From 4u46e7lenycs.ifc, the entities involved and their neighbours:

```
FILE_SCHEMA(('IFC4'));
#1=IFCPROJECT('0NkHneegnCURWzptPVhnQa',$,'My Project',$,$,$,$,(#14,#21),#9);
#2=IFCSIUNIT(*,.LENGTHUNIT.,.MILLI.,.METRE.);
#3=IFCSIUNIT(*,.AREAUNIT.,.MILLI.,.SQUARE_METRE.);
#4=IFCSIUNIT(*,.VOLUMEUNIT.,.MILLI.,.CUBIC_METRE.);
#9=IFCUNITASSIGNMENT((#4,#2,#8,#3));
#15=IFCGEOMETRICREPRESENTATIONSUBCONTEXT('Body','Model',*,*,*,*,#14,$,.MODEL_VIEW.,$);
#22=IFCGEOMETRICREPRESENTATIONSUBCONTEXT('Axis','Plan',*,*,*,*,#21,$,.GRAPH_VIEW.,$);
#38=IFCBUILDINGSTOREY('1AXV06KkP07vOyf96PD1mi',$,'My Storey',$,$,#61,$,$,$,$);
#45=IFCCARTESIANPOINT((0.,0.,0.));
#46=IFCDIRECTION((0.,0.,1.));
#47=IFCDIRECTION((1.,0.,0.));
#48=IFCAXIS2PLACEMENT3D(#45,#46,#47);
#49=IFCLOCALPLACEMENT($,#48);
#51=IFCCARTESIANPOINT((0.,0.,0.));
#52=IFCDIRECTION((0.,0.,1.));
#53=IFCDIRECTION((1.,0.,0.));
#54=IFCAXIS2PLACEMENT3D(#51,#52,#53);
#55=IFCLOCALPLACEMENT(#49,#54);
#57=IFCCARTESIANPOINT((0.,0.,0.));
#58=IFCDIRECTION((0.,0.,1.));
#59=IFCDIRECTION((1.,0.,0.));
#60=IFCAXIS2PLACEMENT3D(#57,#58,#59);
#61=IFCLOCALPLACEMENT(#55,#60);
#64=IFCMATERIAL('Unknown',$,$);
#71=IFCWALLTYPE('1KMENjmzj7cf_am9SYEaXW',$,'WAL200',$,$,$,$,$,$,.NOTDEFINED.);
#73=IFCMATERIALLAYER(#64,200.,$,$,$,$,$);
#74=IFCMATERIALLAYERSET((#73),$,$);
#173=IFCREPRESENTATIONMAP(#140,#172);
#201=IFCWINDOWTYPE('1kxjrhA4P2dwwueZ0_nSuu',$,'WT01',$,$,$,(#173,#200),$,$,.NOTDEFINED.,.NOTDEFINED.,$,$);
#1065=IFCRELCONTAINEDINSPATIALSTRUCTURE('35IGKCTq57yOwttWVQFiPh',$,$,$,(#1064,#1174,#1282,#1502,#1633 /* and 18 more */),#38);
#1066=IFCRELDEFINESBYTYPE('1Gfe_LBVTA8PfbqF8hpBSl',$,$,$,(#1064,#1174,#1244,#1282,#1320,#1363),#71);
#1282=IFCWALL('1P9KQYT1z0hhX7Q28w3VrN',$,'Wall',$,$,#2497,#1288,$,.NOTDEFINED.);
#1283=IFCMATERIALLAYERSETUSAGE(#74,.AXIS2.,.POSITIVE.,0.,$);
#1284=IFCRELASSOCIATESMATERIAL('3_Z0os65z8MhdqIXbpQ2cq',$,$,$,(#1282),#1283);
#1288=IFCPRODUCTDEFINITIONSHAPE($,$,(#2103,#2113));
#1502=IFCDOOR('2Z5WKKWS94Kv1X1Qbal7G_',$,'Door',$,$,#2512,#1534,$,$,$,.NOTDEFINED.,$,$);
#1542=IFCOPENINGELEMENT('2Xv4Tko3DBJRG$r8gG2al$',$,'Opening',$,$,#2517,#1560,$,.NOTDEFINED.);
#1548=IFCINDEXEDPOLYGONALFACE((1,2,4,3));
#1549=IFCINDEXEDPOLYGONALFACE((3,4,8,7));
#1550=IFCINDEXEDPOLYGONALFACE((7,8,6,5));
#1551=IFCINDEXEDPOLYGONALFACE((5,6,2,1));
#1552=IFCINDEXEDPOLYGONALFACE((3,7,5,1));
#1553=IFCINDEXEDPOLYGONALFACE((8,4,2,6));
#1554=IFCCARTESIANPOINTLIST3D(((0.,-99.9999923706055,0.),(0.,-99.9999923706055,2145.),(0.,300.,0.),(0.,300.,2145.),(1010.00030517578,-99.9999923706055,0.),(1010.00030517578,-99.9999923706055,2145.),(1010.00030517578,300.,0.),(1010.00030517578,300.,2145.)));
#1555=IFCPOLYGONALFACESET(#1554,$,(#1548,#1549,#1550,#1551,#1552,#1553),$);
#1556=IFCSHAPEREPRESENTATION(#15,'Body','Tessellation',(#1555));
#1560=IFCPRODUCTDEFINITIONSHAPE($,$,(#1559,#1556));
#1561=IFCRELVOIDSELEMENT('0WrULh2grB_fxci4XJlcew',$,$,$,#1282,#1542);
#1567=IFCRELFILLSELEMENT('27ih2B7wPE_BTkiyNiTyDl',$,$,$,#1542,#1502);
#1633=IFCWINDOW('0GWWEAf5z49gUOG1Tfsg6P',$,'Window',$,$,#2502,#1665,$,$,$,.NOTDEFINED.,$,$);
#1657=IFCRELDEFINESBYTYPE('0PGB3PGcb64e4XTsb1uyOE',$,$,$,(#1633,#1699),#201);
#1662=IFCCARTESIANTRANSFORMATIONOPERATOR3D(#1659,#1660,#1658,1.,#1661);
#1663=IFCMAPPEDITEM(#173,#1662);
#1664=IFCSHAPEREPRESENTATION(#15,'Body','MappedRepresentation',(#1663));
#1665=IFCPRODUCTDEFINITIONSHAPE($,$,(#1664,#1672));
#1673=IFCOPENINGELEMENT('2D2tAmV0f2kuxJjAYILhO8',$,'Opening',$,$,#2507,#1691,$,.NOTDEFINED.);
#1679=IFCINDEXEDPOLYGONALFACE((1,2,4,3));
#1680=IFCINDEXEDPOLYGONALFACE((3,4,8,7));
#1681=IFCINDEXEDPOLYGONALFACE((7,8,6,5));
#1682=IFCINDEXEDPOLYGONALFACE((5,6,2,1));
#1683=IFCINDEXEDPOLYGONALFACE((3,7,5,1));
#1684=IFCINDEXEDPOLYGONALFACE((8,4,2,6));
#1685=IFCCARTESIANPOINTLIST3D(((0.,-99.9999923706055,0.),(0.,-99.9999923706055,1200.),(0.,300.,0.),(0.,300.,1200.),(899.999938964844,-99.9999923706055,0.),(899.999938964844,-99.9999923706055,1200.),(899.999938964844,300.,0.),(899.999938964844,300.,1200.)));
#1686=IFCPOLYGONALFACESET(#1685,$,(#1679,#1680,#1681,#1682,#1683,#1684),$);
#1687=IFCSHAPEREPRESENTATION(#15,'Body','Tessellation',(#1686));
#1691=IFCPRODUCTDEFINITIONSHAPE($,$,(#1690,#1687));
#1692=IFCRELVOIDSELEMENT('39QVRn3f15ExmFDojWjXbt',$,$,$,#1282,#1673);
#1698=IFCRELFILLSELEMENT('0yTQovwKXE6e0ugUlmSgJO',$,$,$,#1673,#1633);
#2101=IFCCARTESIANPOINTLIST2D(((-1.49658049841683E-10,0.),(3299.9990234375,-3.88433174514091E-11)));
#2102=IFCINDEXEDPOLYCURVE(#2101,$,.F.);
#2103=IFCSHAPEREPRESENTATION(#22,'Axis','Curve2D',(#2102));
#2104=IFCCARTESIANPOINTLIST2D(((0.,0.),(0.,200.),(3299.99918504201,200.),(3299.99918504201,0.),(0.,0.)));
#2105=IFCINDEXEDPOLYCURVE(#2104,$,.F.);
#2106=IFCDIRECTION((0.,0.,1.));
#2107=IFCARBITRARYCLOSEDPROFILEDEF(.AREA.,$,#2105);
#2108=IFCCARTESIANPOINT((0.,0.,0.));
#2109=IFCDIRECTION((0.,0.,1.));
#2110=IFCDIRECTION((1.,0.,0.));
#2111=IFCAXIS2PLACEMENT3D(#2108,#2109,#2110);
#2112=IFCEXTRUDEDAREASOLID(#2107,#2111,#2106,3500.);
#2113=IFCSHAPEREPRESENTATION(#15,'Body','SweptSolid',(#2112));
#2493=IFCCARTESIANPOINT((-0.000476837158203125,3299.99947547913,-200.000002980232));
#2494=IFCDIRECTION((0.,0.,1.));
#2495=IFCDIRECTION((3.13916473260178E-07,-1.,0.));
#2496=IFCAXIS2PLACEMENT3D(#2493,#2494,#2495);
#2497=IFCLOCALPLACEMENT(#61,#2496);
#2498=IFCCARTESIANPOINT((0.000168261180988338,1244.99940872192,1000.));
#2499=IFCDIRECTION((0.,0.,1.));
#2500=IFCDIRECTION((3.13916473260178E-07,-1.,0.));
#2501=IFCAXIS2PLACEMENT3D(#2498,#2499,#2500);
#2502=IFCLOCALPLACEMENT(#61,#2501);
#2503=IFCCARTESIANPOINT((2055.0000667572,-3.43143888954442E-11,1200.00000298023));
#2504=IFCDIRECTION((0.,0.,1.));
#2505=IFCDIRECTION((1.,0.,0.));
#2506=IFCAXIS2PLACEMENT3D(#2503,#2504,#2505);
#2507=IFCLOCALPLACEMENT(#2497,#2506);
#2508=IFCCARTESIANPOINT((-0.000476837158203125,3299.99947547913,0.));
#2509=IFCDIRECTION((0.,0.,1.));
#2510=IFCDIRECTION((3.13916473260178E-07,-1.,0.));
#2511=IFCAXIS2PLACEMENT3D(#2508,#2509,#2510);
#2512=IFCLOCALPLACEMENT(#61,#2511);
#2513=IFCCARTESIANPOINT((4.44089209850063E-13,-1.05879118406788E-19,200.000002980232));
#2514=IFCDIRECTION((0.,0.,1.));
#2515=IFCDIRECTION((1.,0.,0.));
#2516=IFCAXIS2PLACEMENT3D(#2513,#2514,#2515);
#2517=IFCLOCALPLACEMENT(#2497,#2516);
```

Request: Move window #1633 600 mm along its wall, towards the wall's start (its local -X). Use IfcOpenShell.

```python
import ifcopenshell
import ifcopenshell.api.geometry
import ifcopenshell.util.placement
import ifcopenshell.util.unit

model = ifcopenshell.open("4u46e7lenycs.ifc")
unit_scale = ifcopenshell.util.unit.calculate_unit_scale(model)

window = model.by_guid("0GWWEAf5z49gUOG1Tfsg6P")
opening = window.FillsVoids[0].RelatingOpeningElement
wall = opening.VoidsElements[0].RelatingBuildingElement

wall_matrix = ifcopenshell.util.placement.get_local_placement(wall.ObjectPlacement)
shift = wall_matrix[:3, 0] * -0.6 / unit_scale
before = ifcopenshell.util.placement.get_local_placement(window.ObjectPlacement)[:3, 3].copy()

# The window is not placed relative to its opening, so move both.
for product in (opening, window):
    matrix = ifcopenshell.util.placement.get_local_placement(product.ObjectPlacement)
    matrix[:3, 3] += shift
    ifcopenshell.api.geometry.edit_object_placement(model, product=product, matrix=matrix, is_si=False)

after = ifcopenshell.util.placement.get_local_placement(window.ObjectPlacement)[:3, 3]
print("window moved by", (after - before).round(3) + 0.0)

model.write("4u46e7lenycs-out.ifc")
```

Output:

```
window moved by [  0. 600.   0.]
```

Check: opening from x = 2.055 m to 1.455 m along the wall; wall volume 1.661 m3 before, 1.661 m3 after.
